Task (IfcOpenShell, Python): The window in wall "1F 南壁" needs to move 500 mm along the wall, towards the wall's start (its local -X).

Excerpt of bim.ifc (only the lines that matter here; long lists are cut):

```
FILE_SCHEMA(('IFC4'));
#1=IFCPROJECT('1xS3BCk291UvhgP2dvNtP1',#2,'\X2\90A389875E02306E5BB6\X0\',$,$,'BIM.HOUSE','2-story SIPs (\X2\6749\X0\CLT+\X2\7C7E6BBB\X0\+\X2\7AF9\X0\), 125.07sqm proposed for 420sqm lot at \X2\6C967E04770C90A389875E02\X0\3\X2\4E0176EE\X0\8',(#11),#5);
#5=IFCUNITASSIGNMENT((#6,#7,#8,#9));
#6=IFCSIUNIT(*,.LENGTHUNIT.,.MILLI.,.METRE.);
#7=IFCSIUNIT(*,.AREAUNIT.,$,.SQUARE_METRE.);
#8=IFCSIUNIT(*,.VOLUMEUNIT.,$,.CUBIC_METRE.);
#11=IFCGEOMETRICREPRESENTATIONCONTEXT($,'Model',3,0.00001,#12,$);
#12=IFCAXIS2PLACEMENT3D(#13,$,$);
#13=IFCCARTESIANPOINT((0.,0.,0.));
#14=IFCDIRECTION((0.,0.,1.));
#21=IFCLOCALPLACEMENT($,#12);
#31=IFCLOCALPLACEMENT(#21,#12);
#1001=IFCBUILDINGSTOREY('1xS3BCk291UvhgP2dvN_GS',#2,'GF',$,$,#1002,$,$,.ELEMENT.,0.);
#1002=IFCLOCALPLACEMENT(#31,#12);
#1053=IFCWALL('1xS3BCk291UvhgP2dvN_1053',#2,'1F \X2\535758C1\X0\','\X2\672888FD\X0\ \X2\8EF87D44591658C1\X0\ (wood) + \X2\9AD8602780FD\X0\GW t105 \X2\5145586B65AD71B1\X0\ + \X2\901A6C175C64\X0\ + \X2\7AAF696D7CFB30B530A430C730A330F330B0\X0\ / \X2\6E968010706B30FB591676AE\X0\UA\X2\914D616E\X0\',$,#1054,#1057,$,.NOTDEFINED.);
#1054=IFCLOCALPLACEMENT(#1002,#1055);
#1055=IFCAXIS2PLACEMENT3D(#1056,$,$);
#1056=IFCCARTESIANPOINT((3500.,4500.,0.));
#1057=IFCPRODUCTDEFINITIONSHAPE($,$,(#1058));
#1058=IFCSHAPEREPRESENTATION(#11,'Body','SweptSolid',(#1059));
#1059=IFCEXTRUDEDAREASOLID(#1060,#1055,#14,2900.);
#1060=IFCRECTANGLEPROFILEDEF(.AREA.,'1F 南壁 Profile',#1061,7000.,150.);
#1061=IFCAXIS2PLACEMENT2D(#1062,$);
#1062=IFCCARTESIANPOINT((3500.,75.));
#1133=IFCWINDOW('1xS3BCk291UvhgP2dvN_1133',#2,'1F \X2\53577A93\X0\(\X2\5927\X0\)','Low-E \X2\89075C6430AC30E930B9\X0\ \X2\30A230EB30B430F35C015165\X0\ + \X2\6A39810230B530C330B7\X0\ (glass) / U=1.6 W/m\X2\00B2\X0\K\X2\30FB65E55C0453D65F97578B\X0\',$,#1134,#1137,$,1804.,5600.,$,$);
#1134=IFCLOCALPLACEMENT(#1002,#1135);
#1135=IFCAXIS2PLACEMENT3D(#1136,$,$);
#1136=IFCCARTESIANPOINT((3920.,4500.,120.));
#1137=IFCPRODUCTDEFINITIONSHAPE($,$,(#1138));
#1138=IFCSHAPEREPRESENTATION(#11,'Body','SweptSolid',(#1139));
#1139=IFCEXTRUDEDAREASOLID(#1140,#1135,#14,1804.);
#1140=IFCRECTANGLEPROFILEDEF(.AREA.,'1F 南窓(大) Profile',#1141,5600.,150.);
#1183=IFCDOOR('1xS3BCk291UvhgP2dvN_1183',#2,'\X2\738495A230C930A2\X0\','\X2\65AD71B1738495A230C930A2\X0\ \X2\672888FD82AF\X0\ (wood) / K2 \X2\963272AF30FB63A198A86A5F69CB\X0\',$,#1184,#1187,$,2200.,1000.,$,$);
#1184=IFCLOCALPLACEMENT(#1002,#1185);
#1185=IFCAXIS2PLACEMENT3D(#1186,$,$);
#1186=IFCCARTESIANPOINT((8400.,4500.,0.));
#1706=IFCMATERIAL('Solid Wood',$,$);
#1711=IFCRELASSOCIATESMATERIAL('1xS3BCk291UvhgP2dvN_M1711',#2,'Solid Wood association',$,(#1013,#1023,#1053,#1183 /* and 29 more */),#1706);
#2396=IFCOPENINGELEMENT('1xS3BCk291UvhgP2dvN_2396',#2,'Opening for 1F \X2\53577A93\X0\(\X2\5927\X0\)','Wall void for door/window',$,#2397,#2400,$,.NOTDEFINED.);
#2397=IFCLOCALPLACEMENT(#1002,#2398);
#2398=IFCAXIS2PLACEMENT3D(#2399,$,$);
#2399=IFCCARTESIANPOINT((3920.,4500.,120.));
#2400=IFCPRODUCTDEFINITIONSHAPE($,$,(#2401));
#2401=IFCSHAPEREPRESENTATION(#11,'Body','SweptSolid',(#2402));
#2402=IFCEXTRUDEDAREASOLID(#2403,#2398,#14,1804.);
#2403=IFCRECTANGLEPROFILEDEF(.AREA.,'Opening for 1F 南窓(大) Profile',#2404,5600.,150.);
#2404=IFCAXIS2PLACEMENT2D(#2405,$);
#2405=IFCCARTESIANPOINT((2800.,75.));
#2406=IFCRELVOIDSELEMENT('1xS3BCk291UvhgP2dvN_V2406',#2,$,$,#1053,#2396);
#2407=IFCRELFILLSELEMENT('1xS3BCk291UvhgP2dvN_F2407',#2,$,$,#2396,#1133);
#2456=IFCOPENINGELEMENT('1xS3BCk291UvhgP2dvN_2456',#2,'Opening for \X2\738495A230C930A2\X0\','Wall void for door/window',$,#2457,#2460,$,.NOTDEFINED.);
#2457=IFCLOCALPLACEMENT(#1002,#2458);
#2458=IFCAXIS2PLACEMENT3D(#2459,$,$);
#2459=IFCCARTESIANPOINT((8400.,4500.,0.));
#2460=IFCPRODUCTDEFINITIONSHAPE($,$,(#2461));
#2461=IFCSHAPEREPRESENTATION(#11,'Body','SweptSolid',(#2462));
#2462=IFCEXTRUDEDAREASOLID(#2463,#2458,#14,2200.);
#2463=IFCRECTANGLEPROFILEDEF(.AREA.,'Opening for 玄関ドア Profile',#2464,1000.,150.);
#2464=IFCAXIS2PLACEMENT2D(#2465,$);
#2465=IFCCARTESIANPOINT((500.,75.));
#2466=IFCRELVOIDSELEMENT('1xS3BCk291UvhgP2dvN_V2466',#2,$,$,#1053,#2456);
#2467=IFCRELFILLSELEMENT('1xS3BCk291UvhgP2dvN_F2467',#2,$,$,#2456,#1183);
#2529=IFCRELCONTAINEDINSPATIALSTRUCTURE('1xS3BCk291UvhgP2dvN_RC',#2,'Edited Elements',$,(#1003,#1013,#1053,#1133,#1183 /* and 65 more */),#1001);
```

```python
import ifcopenshell
import ifcopenshell.api.geometry
import ifcopenshell.util.placement
import ifcopenshell.util.unit

model = ifcopenshell.open("bim.ifc")
unit_scale = ifcopenshell.util.unit.calculate_unit_scale(model)

window = model.by_guid("1xS3BCk291UvhgP2dvN_1133")
opening = window.FillsVoids[0].RelatingOpeningElement
wall = opening.VoidsElements[0].RelatingBuildingElement

wall_matrix = ifcopenshell.util.placement.get_local_placement(wall.ObjectPlacement)
shift = wall_matrix[:3, 0] * -0.5 / unit_scale
before = ifcopenshell.util.placement.get_local_placement(window.ObjectPlacement)[:3, 3].copy()

# The window is not placed relative to its opening, so move both.
for product in (opening, window):
    matrix = ifcopenshell.util.placement.get_local_placement(product.ObjectPlacement)
    matrix[:3, 3] += shift
    ifcopenshell.api.geometry.edit_object_placement(model, product=product, matrix=matrix, is_si=False)

after = ifcopenshell.util.placement.get_local_placement(window.ObjectPlacement)[:3, 3]
print("window moved by", (after - before).round(3) + 0.0)

model.write("bim_updated.ifc")
```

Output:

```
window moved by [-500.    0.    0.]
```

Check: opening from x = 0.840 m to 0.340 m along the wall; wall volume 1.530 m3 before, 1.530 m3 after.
